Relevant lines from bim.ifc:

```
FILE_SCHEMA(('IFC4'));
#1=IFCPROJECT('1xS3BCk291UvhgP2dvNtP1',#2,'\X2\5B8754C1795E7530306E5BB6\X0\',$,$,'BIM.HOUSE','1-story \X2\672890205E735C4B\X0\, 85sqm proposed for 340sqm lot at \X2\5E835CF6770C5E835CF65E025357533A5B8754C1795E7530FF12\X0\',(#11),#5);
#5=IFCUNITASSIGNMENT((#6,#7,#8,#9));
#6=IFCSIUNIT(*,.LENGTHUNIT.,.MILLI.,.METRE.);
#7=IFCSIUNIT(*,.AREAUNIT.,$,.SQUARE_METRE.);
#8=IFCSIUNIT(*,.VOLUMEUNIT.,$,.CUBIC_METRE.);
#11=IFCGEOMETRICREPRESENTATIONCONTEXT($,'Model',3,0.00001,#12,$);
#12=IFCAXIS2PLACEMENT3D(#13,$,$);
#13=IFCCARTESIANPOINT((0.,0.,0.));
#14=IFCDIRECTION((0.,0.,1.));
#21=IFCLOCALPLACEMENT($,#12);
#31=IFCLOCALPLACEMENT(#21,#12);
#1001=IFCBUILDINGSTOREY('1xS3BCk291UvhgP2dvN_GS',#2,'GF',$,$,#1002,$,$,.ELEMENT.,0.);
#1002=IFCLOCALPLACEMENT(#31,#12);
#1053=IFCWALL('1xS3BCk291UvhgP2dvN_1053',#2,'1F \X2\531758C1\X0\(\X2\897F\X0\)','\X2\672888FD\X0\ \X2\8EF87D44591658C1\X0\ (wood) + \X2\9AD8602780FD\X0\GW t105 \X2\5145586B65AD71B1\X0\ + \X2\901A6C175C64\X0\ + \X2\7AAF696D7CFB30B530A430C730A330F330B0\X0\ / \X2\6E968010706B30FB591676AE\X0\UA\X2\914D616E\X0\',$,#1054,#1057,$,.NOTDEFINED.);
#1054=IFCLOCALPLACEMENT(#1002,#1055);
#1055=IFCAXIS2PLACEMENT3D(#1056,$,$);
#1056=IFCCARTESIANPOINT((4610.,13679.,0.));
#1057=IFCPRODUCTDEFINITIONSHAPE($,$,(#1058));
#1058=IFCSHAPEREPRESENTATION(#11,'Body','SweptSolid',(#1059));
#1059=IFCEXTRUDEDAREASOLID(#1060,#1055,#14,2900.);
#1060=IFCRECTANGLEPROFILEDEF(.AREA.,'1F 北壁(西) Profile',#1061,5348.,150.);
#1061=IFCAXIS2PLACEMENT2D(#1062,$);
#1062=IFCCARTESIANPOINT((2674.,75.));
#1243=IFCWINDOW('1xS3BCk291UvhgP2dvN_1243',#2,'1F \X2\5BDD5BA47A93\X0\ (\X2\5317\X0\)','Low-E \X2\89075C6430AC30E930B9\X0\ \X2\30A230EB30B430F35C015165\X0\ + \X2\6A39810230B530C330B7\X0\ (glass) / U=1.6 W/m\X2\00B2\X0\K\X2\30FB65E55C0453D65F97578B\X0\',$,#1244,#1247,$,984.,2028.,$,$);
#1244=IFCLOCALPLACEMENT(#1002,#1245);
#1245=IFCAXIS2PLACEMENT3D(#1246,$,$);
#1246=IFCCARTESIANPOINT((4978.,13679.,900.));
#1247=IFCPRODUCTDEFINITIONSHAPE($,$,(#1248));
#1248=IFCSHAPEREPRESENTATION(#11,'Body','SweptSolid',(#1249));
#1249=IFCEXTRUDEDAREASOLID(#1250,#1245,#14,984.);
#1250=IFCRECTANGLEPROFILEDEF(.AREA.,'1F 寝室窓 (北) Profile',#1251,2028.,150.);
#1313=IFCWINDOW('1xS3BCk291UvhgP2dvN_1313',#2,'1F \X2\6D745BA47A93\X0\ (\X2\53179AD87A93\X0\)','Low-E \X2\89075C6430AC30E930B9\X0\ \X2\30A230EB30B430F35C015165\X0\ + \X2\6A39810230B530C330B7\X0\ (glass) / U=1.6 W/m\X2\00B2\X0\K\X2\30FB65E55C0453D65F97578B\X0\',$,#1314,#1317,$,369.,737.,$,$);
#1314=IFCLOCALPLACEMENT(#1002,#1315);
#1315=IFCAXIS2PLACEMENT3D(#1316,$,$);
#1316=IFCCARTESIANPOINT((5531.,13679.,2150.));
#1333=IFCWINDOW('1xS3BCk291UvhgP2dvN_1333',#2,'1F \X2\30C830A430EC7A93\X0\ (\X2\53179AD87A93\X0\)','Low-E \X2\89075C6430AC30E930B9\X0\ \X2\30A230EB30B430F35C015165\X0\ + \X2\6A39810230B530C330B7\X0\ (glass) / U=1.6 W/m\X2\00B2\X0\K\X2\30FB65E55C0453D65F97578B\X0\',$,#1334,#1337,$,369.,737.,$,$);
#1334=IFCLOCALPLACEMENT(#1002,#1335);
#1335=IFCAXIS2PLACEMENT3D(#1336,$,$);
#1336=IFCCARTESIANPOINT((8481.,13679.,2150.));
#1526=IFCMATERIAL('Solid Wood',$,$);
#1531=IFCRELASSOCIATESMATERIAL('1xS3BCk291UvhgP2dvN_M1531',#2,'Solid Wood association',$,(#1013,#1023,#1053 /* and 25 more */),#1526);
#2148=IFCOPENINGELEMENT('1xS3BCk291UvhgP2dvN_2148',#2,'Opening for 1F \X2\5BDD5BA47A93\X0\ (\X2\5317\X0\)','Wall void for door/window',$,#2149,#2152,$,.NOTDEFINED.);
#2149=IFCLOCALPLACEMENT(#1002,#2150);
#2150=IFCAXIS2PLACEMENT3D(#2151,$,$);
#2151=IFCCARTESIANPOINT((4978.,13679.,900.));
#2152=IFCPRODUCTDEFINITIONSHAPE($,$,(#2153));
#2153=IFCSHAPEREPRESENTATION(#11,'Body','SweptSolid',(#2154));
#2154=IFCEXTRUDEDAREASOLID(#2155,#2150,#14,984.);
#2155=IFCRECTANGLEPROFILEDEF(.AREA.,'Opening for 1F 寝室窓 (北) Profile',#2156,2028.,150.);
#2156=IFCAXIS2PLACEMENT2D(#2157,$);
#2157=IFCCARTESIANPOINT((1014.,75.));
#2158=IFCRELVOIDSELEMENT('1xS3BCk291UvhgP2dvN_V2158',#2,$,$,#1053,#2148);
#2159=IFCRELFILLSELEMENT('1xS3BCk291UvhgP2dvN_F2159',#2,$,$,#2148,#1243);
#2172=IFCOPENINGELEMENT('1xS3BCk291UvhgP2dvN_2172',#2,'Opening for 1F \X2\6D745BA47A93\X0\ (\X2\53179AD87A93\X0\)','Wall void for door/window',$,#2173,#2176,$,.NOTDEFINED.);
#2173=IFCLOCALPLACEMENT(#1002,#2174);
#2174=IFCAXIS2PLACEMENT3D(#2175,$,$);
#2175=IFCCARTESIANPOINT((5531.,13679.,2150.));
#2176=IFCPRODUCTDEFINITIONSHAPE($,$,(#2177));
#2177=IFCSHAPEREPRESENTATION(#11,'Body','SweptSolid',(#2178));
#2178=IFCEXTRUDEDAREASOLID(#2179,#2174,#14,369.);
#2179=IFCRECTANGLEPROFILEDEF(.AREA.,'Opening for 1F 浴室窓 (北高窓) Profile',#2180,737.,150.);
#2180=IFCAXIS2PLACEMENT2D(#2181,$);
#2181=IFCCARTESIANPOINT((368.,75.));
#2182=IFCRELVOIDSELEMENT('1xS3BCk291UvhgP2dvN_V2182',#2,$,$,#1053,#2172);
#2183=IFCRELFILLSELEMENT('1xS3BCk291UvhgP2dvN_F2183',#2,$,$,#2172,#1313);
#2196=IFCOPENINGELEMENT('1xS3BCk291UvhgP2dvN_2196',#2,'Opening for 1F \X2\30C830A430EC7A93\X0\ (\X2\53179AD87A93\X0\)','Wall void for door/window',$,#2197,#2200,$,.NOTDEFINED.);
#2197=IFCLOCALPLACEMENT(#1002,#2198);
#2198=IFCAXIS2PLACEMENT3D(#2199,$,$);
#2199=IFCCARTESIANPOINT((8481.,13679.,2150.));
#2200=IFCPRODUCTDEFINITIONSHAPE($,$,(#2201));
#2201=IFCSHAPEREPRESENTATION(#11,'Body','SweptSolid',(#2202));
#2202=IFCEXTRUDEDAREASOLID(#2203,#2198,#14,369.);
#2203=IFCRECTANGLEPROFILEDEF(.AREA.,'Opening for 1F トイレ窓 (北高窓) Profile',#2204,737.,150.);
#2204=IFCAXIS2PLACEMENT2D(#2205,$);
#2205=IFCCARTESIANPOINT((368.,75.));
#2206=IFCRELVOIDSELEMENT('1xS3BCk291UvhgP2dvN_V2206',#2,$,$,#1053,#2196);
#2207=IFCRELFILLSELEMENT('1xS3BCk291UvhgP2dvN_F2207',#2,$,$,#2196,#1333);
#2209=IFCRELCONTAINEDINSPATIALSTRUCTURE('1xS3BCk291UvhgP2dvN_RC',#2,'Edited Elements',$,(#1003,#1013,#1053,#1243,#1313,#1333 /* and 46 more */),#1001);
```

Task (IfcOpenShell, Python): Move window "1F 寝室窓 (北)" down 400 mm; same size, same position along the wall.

```python
import numpy as np
import ifcopenshell
import ifcopenshell.api.geometry
import ifcopenshell.util.placement
import ifcopenshell.util.unit

model = ifcopenshell.open("bim.ifc")
unit_scale = ifcopenshell.util.unit.calculate_unit_scale(model)

window = model.by_guid("1xS3BCk291UvhgP2dvN_1243")
opening = window.FillsVoids[0].RelatingOpeningElement
dz = -0.4 / unit_scale

shift = np.array([0.0, 0.0, dz])
# The window is not placed relative to its opening, so move both.
for product in (opening, window):
    matrix = ifcopenshell.util.placement.get_local_placement(product.ObjectPlacement)
    matrix[:3, 3] += shift
    ifcopenshell.api.geometry.edit_object_placement(model, product=product, matrix=matrix, is_si=False)

print(f"moved by {dz * unit_scale:+.3f} m")

model.write("bim_rev.ifc")
```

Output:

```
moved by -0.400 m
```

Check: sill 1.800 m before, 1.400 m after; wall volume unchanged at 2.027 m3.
